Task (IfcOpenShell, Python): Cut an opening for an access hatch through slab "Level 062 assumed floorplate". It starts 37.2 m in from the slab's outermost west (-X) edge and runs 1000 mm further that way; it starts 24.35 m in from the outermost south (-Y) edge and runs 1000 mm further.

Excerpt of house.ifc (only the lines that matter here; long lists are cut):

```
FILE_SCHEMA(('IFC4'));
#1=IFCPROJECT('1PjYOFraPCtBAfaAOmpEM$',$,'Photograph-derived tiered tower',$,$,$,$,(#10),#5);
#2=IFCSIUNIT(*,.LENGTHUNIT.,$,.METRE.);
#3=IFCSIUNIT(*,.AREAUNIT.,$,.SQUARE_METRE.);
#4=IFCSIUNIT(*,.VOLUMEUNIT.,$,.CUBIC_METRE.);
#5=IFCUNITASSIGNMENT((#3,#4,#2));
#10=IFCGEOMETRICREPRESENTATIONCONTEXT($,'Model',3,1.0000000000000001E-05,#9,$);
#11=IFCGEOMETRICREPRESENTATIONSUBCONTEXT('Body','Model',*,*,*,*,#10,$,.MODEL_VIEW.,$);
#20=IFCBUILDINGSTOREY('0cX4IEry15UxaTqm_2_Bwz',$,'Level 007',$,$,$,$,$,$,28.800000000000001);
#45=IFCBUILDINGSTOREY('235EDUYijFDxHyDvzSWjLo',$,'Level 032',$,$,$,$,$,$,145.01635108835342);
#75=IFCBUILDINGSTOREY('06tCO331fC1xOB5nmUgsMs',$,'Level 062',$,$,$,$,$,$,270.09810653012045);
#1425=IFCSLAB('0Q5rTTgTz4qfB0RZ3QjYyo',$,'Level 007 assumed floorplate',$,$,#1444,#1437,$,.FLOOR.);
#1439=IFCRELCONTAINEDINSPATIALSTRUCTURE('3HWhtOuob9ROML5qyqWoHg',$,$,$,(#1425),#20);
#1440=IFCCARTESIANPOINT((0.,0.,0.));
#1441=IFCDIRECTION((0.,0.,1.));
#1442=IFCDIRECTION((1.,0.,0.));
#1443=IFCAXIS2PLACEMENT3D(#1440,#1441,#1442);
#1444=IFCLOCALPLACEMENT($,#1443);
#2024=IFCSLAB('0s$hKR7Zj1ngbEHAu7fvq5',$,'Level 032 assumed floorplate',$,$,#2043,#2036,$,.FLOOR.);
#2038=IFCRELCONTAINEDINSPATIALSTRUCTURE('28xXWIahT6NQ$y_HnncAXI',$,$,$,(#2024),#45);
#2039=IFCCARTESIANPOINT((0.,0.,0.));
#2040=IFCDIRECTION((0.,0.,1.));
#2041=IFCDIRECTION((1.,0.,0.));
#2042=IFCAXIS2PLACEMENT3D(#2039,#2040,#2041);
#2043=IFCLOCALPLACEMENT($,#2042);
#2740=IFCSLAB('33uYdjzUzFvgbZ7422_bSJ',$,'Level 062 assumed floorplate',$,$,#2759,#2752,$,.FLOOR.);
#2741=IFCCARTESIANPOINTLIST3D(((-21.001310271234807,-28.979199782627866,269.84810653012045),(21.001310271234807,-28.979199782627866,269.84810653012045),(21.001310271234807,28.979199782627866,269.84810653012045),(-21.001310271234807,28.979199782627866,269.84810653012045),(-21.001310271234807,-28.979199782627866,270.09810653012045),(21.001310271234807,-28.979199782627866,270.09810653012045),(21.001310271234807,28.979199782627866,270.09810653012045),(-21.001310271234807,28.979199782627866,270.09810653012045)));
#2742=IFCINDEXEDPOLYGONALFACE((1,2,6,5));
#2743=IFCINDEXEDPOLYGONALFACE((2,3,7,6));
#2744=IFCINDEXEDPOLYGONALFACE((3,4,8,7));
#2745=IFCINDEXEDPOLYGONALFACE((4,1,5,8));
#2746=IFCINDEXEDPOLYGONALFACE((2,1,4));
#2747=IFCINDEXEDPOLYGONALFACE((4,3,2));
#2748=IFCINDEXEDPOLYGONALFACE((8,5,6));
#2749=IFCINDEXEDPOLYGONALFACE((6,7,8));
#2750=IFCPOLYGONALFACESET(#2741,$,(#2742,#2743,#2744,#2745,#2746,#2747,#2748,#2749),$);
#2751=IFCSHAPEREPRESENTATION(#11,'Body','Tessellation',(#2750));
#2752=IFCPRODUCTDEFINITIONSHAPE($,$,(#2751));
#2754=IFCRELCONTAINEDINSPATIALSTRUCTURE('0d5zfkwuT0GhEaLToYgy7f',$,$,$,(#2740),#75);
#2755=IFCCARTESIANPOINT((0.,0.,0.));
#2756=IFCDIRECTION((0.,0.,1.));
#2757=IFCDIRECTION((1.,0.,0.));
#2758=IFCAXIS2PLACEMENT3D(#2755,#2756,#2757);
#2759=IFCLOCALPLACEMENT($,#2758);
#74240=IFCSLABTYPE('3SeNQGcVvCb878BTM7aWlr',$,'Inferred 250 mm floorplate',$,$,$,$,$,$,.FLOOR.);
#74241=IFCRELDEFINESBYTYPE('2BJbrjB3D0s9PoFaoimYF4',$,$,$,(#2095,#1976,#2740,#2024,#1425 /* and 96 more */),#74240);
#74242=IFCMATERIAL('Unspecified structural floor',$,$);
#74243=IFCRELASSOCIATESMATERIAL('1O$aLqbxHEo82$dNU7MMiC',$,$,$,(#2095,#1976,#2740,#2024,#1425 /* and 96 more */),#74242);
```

```python
import numpy as np
import ifcopenshell
import ifcopenshell.api.feature
import ifcopenshell.api.geometry
import ifcopenshell.api.root
import ifcopenshell.geom
import ifcopenshell.util.placement
import ifcopenshell.util.representation
import ifcopenshell.util.shape
import ifcopenshell.util.unit

model = ifcopenshell.open("house.ifc")
unit_scale = ifcopenshell.util.unit.calculate_unit_scale(model)
settings = ifcopenshell.geom.settings()


def volume(element):
    """Net volume in cubic metres, openings subtracted."""
    shape = ifcopenshell.geom.create_shape(settings, element)
    return ifcopenshell.util.shape.get_volume(shape.geometry)


slab = model.by_guid("33uYdjzUzFvgbZ7422_bSJ")
before = volume(slab)

# Extent in the slab's own axes, in metres. The edges named are its -X and -Y sides.
slab_shape = ifcopenshell.geom.create_shape(settings, slab)
vertices = ifcopenshell.util.shape.get_vertices(slab_shape.geometry)
x_min, y_min, bottom = vertices.min(axis=0)
top = vertices[:, 2].max()

opening = ifcopenshell.api.root.create_entity(model, ifc_class="IfcOpeningElement", name="Access hatch opening", predefined_type="OPENING")
context = ifcopenshell.util.representation.get_context(model, "Model", "Body", "MODEL_VIEW")
width, depth = 1, 1
outline = [(0.0, 0.0), (width, 0.0), (width, depth), (0.0, depth), (0.0, 0.0)]
# Overshoot both faces by 50 mm so the cut is clean.
shape = ifcopenshell.api.geometry.add_slab_representation(
    model, context=context, depth=top - bottom + 0.1, polyline=outline
)
ifcopenshell.api.geometry.assign_representation(model, product=opening, representation=shape)

matrix = ifcopenshell.util.placement.get_local_placement(slab.ObjectPlacement)
matrix[:, 3] = matrix @ np.append(np.array([x_min + 37.2, y_min + 24.35, bottom - 0.05]) / unit_scale, 1.0)
ifcopenshell.api.geometry.edit_object_placement(model, product=opening, matrix=matrix, is_si=False)
ifcopenshell.api.feature.add_feature(model, feature=opening, element=slab)

after = volume(slab)

print(f"slab volume {before:.3f} -> {after:.3f} m3")

model.write("house_rev.ifc")
```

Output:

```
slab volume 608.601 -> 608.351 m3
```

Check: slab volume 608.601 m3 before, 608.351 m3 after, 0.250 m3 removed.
